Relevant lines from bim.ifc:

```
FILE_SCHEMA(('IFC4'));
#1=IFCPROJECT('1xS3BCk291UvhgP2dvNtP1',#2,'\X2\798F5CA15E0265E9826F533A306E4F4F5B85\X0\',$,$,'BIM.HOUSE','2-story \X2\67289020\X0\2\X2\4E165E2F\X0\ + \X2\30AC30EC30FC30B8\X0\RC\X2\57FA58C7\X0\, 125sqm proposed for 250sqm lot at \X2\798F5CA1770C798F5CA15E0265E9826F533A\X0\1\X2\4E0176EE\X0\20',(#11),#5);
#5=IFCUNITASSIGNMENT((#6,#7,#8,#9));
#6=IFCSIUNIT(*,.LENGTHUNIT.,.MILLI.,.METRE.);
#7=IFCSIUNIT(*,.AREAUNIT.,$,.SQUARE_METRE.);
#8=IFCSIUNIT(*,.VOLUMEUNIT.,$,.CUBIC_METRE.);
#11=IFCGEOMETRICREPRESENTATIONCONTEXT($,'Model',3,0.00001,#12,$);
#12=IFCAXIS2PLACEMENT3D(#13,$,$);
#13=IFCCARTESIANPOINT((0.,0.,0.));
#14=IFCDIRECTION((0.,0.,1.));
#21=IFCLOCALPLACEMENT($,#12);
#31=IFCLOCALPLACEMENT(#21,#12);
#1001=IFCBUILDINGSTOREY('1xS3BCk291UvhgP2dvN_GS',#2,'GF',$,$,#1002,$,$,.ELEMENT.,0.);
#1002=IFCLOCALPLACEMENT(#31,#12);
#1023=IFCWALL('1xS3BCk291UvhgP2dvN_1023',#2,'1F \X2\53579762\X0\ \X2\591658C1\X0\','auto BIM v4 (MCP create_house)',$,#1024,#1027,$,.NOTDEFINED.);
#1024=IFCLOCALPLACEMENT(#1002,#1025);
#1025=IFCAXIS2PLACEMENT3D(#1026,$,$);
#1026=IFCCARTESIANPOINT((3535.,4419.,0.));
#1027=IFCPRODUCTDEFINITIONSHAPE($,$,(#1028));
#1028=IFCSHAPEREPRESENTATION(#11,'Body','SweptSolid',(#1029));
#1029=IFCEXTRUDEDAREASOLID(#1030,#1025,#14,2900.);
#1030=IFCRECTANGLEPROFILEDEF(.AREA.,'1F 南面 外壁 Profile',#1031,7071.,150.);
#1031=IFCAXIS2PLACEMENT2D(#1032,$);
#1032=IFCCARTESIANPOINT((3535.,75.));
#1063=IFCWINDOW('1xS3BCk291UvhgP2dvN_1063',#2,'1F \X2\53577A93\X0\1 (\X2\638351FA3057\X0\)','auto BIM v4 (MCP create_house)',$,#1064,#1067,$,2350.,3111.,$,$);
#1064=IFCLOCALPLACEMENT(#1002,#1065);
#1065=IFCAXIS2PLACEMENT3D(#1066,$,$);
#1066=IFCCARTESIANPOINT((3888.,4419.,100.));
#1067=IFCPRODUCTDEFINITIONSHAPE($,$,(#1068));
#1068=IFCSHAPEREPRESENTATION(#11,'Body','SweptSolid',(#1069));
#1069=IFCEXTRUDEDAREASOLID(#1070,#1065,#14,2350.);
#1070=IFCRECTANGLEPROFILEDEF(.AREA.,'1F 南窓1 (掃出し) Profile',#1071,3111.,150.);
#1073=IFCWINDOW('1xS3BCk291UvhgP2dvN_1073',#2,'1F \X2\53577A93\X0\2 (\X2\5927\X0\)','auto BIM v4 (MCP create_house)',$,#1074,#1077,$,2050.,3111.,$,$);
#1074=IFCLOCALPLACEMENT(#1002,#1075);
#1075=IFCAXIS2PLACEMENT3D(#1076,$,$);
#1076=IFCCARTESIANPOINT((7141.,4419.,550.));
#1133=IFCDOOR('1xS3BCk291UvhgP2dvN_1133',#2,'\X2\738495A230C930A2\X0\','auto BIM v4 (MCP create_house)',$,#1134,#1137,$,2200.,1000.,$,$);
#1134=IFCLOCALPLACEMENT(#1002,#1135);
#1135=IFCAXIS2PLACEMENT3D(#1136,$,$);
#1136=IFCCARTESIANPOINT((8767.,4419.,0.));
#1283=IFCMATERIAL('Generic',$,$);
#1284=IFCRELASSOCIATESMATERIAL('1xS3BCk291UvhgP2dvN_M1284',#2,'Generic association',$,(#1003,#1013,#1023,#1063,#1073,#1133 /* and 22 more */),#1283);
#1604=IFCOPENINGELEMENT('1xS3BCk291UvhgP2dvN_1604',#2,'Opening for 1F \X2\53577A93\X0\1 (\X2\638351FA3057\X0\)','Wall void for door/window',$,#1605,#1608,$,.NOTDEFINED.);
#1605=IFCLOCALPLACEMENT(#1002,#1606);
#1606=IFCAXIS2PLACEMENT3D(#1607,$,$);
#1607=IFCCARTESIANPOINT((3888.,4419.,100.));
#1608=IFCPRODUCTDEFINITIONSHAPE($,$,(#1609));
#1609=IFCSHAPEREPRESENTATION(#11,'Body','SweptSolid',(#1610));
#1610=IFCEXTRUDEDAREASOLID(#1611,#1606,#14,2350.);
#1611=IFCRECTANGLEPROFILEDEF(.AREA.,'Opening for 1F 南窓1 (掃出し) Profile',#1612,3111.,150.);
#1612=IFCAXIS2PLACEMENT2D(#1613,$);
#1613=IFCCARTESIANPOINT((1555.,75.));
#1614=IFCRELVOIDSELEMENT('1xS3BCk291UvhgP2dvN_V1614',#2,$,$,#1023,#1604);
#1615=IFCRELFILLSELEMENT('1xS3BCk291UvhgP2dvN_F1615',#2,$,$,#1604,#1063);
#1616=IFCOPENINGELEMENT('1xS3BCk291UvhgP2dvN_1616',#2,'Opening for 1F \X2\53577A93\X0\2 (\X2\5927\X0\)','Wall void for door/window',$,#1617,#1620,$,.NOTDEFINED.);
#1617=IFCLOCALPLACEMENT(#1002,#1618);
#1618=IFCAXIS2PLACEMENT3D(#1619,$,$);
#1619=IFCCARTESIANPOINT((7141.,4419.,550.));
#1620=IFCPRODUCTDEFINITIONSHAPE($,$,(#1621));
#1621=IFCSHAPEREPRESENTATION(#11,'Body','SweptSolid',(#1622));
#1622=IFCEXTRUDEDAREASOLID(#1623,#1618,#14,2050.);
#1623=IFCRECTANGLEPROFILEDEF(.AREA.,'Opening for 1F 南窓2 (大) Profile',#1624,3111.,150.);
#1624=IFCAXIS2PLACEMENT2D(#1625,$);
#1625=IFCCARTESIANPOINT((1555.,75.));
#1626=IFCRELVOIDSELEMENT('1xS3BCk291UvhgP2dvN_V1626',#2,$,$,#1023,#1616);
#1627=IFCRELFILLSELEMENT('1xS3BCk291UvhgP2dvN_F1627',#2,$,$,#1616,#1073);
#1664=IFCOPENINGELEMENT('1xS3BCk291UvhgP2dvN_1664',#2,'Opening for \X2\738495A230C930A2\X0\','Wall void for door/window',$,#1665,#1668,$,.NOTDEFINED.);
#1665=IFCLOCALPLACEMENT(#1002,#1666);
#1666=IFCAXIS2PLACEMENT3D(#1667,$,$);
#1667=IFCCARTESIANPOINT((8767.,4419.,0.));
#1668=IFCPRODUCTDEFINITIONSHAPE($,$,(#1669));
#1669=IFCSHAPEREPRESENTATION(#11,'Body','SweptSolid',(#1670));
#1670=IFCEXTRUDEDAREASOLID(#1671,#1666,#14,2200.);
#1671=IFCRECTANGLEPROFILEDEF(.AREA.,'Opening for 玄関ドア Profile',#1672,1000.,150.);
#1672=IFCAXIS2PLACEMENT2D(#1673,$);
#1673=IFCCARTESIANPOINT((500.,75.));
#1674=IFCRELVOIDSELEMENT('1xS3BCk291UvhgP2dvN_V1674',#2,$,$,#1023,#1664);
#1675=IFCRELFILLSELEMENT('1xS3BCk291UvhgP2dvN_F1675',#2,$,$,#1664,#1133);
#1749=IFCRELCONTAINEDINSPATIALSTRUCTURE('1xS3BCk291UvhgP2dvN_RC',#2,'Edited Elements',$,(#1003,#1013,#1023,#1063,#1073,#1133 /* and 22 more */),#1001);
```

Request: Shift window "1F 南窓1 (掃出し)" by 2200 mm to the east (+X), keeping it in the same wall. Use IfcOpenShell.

```python
import ifcopenshell
import ifcopenshell.api.geometry
import ifcopenshell.util.placement
import ifcopenshell.util.unit

model = ifcopenshell.open("bim.ifc")
unit_scale = ifcopenshell.util.unit.calculate_unit_scale(model)

window = model.by_guid("1xS3BCk291UvhgP2dvN_1063")
opening = window.FillsVoids[0].RelatingOpeningElement
wall = opening.VoidsElements[0].RelatingBuildingElement

wall_matrix = ifcopenshell.util.placement.get_local_placement(wall.ObjectPlacement)
shift = wall_matrix[:3, 0] * 2.2 / unit_scale
before = ifcopenshell.util.placement.get_local_placement(window.ObjectPlacement)[:3, 3].copy()

# The window is not placed relative to its opening, so move both.
for product in (opening, window):
    matrix = ifcopenshell.util.placement.get_local_placement(product.ObjectPlacement)
    matrix[:3, 3] += shift
    ifcopenshell.api.geometry.edit_object_placement(model, product=product, matrix=matrix, is_si=False)

after = ifcopenshell.util.placement.get_local_placement(window.ObjectPlacement)[:3, 3]
print("window moved by", (after - before).round(3) + 0.0)

model.write("bim-out.ifc")
```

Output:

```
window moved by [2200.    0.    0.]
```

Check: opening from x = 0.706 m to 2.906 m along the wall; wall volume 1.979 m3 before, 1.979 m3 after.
